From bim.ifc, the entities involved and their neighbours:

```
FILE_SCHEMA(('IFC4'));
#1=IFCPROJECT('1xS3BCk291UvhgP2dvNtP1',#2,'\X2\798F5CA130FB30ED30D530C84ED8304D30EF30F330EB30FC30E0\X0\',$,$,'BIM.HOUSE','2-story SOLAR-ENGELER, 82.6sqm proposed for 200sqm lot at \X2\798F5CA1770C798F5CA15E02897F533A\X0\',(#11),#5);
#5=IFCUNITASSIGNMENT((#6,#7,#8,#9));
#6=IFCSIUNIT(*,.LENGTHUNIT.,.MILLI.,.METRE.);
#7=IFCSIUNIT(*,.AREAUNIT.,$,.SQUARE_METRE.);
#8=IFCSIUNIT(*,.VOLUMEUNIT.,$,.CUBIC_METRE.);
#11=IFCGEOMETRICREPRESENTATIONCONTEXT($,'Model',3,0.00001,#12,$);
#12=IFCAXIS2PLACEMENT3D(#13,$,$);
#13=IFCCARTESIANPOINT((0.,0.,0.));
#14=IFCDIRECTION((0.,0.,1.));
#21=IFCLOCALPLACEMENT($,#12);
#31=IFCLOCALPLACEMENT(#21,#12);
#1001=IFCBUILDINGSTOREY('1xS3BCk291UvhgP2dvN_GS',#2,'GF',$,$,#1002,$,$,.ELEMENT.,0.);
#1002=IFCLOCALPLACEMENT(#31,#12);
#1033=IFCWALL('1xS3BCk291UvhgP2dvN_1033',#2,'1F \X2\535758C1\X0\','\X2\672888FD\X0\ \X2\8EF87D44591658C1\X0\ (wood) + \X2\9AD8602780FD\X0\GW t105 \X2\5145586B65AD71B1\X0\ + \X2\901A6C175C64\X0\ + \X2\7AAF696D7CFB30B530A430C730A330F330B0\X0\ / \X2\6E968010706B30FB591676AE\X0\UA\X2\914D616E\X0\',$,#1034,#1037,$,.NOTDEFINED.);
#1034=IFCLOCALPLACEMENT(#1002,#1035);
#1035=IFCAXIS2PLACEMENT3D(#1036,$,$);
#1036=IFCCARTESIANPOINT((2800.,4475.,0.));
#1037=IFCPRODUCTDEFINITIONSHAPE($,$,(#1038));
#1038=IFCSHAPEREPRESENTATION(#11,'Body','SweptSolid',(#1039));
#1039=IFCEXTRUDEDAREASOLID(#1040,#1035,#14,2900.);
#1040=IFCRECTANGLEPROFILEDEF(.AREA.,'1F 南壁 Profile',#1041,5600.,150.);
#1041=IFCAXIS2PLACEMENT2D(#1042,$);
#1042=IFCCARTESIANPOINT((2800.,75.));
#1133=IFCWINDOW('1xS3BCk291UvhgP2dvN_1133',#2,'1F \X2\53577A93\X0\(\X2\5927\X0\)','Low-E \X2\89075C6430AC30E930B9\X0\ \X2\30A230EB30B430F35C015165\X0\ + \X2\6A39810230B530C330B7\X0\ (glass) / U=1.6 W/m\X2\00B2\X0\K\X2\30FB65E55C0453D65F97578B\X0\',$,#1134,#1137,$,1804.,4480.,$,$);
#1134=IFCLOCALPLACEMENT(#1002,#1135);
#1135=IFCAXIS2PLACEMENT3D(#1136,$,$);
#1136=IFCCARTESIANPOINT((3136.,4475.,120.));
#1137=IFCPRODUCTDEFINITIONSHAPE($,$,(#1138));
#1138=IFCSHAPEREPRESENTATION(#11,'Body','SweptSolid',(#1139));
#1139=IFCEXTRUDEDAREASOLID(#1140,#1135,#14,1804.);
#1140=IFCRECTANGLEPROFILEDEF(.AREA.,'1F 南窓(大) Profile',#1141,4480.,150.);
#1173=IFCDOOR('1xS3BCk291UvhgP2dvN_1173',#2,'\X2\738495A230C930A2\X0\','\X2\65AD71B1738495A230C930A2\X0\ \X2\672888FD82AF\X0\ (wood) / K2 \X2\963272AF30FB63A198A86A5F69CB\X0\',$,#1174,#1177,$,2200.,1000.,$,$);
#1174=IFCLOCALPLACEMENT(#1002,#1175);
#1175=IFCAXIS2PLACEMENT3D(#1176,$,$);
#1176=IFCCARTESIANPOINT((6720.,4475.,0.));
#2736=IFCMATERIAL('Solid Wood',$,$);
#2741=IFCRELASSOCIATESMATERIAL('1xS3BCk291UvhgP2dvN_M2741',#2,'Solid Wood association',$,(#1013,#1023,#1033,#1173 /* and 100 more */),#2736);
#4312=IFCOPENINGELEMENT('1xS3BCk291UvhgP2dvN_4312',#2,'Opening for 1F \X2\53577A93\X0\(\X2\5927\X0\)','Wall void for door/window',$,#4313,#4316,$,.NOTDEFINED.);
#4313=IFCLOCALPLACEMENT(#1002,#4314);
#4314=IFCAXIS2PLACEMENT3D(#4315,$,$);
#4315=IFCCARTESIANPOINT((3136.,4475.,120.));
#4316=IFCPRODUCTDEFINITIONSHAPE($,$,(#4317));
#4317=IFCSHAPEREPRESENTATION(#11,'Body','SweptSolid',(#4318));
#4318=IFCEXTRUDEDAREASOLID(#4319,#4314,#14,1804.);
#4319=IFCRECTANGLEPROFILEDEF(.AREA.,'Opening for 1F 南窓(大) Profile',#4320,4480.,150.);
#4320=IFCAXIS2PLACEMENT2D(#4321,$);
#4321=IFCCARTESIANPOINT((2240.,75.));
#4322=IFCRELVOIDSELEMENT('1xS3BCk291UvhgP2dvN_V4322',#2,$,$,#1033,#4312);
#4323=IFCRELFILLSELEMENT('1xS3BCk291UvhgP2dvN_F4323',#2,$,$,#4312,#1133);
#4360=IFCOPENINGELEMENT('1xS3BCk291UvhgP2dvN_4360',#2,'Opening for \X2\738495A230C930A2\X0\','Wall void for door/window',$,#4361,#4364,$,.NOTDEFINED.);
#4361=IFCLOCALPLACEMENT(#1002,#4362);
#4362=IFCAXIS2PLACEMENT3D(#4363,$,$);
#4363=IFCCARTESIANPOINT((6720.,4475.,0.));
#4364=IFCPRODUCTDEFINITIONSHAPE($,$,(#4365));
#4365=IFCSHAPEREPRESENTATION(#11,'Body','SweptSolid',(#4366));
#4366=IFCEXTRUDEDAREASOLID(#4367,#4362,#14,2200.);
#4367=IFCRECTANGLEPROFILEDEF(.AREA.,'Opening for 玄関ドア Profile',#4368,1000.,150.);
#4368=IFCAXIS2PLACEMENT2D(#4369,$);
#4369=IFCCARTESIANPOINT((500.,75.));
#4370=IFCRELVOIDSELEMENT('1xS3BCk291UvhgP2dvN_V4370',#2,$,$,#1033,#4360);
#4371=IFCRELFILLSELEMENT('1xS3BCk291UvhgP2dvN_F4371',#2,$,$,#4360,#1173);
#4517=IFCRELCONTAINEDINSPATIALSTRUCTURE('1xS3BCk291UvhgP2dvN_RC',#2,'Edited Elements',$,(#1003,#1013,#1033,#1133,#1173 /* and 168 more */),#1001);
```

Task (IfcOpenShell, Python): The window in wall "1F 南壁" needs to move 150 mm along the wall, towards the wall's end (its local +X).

```python
import ifcopenshell
import ifcopenshell.api.geometry
import ifcopenshell.util.placement
import ifcopenshell.util.unit

model = ifcopenshell.open("bim.ifc")
unit_scale = ifcopenshell.util.unit.calculate_unit_scale(model)

window = model.by_guid("1xS3BCk291UvhgP2dvN_1133")
opening = window.FillsVoids[0].RelatingOpeningElement
wall = opening.VoidsElements[0].RelatingBuildingElement

wall_matrix = ifcopenshell.util.placement.get_local_placement(wall.ObjectPlacement)
shift = wall_matrix[:3, 0] * 0.15 / unit_scale
before = ifcopenshell.util.placement.get_local_placement(window.ObjectPlacement)[:3, 3].copy()

# The window is not placed relative to its opening, so move both.
for product in (opening, window):
    matrix = ifcopenshell.util.placement.get_local_placement(product.ObjectPlacement)
    matrix[:3, 3] += shift
    ifcopenshell.api.geometry.edit_object_placement(model, product=product, matrix=matrix, is_si=False)

after = ifcopenshell.util.placement.get_local_placement(window.ObjectPlacement)[:3, 3]
print("window moved by", (after - before).round(3) + 0.0)

model.write("bim_edited.ifc")
```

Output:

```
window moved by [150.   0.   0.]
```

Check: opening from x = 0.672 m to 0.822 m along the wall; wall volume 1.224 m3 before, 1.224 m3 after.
